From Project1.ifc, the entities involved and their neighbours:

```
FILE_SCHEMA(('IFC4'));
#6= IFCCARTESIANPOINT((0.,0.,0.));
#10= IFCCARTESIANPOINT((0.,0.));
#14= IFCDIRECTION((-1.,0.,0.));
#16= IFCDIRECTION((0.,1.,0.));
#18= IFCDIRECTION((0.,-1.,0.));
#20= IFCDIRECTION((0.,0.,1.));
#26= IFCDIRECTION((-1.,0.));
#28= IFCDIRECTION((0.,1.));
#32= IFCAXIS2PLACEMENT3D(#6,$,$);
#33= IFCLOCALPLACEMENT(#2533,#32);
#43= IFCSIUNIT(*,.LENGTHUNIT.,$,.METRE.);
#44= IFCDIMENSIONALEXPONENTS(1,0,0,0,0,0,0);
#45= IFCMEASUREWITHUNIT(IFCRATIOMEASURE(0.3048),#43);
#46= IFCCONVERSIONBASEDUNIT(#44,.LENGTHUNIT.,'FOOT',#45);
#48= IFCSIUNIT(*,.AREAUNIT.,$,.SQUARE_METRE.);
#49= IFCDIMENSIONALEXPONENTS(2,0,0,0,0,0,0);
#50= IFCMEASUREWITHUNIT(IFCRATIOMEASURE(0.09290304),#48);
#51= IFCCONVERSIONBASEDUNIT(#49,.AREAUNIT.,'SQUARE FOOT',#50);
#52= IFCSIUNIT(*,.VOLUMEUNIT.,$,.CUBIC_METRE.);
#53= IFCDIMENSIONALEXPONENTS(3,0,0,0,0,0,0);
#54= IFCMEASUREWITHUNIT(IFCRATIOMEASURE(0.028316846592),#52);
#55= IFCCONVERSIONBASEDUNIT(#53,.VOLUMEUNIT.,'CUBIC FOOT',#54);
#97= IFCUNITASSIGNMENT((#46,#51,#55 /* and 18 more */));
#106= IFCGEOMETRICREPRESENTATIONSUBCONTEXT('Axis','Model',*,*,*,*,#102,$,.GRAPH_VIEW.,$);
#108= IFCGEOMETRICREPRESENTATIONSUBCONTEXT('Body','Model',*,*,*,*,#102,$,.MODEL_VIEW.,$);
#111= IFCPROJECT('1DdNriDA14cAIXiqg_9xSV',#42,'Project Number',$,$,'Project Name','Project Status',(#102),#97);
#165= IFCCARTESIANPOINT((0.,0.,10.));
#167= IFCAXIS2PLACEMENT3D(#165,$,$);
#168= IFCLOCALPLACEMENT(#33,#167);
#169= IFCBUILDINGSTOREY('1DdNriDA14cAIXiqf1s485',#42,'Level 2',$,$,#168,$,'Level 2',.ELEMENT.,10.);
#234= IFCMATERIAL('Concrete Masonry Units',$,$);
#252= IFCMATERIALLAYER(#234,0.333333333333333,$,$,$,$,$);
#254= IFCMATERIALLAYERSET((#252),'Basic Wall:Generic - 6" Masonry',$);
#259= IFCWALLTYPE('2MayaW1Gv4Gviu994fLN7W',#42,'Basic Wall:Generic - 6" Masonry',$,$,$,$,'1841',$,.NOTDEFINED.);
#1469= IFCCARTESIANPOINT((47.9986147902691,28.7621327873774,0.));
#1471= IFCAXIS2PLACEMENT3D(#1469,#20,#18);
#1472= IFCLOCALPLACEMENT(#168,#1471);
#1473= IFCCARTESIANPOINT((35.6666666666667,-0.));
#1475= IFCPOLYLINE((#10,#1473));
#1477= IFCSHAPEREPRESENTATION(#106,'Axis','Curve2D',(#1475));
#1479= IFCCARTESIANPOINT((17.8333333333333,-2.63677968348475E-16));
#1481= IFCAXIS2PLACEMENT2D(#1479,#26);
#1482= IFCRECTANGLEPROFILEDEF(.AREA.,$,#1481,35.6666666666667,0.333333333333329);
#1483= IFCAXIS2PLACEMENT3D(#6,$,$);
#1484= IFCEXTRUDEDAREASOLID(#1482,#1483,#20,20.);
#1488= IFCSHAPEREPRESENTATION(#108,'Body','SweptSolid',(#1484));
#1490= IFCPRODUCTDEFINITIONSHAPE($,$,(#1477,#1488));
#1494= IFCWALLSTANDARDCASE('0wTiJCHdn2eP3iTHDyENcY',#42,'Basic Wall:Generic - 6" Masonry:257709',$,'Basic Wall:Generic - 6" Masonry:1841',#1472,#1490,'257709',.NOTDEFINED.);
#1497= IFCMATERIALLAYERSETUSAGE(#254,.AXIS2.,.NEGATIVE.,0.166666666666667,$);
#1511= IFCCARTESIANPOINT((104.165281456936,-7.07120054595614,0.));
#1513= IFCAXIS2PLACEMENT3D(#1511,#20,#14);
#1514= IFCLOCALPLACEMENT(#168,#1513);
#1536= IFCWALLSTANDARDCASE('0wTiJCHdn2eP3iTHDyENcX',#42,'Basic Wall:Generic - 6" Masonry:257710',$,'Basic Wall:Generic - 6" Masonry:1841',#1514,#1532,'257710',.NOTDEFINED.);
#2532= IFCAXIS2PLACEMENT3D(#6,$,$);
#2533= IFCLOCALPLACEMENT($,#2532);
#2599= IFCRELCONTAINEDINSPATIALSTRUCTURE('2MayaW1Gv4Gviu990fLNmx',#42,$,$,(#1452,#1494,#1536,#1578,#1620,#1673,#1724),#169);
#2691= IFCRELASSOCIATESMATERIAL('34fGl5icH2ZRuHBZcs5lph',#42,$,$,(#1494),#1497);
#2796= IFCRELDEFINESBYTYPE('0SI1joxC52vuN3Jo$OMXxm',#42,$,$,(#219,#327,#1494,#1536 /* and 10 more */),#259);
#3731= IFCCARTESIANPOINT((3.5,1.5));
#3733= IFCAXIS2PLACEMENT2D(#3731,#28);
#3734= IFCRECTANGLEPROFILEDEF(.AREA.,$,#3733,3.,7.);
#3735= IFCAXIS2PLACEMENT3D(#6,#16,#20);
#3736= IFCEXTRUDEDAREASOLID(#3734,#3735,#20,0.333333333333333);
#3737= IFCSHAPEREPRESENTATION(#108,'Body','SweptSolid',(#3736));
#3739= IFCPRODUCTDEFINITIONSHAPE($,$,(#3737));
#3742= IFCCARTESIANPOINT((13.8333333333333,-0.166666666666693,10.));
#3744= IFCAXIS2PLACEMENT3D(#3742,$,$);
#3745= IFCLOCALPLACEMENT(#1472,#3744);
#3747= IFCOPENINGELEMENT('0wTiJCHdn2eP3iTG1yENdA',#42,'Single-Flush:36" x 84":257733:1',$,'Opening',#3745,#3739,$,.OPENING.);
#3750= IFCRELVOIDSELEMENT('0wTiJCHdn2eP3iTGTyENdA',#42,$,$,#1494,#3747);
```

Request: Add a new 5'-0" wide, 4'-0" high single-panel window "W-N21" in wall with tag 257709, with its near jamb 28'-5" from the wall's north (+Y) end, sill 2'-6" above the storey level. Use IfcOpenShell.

```python
import numpy as np
import ifcopenshell
import ifcopenshell.api.feature
import ifcopenshell.api.geometry
import ifcopenshell.api.root
import ifcopenshell.api.spatial
import ifcopenshell.geom
import ifcopenshell.util.element
import ifcopenshell.util.placement
import ifcopenshell.util.representation
import ifcopenshell.util.shape
import ifcopenshell.util.unit

model = ifcopenshell.open("Project1.ifc")
unit_scale = ifcopenshell.util.unit.calculate_unit_scale(model)
settings = ifcopenshell.geom.settings()


def volume(element):
    """Net volume in cubic metres, openings subtracted."""
    shape = ifcopenshell.geom.create_shape(settings, element)
    return ifcopenshell.util.shape.get_volume(shape.geometry)


wall = model.by_id(1494)
storey = ifcopenshell.util.element.get_container(wall, ifc_class="IfcBuildingStorey")
context = ifcopenshell.util.representation.get_context(model, "Model", "Body", "MODEL_VIEW")
before = volume(wall)

width, height, from_end, sill = 1.524, 1.2192, 8.6614, 0.762  # metres

# The wall runs along its own X axis, and the end named is its -X end.
wall_shape = ifcopenshell.geom.create_shape(settings, wall)
x, y, z = ifcopenshell.util.shape.get_vertices(wall_shape.geometry).T
start = x.min() + from_end
face, thickness = float(y.min()), float(y.max() - y.min())
wall_matrix = ifcopenshell.util.placement.get_local_placement(wall.ObjectPlacement)
level = ifcopenshell.util.placement.get_local_placement(storey.ObjectPlacement)[2, 3]


def in_wall(x, y):
    """Placement at x, y metres in the wall's axes, at sill height."""
    matrix = wall_matrix.copy()
    matrix[:, 3] = wall_matrix @ np.array([x / unit_scale, y / unit_scale, 0.0, 1.0])
    matrix[2, 3] = level + sill / unit_scale
    return matrix


# Opening: a box that overshoots both wall faces by 50 mm.
opening = ifcopenshell.api.root.create_entity(model, ifc_class="IfcOpeningElement", predefined_type="OPENING")
box = ifcopenshell.api.geometry.add_wall_representation(
    model, context=context, length=width, height=height, thickness=thickness + 0.1
)
ifcopenshell.api.geometry.assign_representation(model, product=opening, representation=box)
ifcopenshell.api.geometry.edit_object_placement(model, product=opening, matrix=in_wall(start, face - 0.05), is_si=False)
ifcopenshell.api.feature.add_feature(model, feature=opening, element=wall)

window = ifcopenshell.api.root.create_entity(model, ifc_class="IfcWindow", name="W-N21", predefined_type="WINDOW")
window.OverallWidth, window.OverallHeight = width / unit_scale, height / unit_scale
window.PartitioningType = "SINGLE_PANEL"
body = ifcopenshell.api.geometry.add_window_representation(
    model,
    context=context,
    overall_width=window.OverallWidth,
    overall_height=window.OverallHeight,
    partition_type="SINGLE_PANEL",
)
ifcopenshell.api.geometry.assign_representation(model, product=window, representation=body)
ifcopenshell.api.spatial.assign_container(model, products=[window], relating_structure=storey)
ifcopenshell.api.feature.add_filling(model, opening=opening, element=window)

# Centre the window in the wall's thickness.
ifcopenshell.api.geometry.edit_object_placement(model, product=window, matrix=in_wall(start, face), is_si=False)
window_shape = ifcopenshell.geom.create_shape(settings, window)
depth = ifcopenshell.util.shape.get_vertices(window_shape.geometry)[:, 1]
offset = face + thickness / 2 - (depth.min() + depth.max()) / 2
ifcopenshell.api.geometry.edit_object_placement(model, product=window, matrix=in_wall(start, offset), is_si=False)

after = volume(wall)

print(f"wall volume {before:.3f} -> {after:.3f} m3")

model.write("Project1-out.ifc")
```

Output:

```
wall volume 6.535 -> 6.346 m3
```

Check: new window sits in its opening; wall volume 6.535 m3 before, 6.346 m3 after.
